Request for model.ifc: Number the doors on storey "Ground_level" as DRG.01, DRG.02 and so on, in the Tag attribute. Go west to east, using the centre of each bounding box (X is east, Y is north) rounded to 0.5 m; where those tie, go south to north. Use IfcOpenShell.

First a look at what the model holds.

```python
import ifcopenshell
import ifcopenshell.util.element
import ifcopenshell.util.placement

model = ifcopenshell.open("model.ifc")
print(model.schema)
storey = next(s for s in model.by_type("IfcBuildingStorey") if s.Name == "Ground_level")
doors = [e for e in ifcopenshell.util.element.get_decomposition(storey) if e.is_a("IfcDoor")]
for e in sorted(doors, key=lambda e: e.id()):
    origin = ifcopenshell.util.placement.get_local_placement(e.ObjectPlacement)[:3, 3]
    print(e.id(), e.Tag, e.Name, origin.round(2) + 0.0, sep=" | ")
```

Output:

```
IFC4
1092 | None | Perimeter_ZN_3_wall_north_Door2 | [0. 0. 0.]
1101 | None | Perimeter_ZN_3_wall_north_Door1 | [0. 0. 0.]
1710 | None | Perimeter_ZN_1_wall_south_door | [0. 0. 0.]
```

```python
import ifcopenshell
import ifcopenshell.geom
import ifcopenshell.util.element
import ifcopenshell.util.shape

model = ifcopenshell.open("model.ifc")
settings = ifcopenshell.geom.settings()
settings.set("use-world-coords", True)


def centre(element):
    shape = ifcopenshell.geom.create_shape(settings, element)
    return ifcopenshell.util.shape.get_bbox_centroid(shape.geometry)


storey = next(s for s in model.by_type("IfcBuildingStorey") if s.Name == "Ground_level")
doors = [e for e in ifcopenshell.util.element.get_decomposition(storey) if e.is_a("IfcDoor")]

# Insertion points can sit at a corner or the storey origin, so sort by the geometry (in metres).
centres = {e: centre(e) for e in doors}
doors.sort(key=lambda e: (round(centres[e][0] / 0.5), centres[e][1]))

for i, e in enumerate(doors, start=1):
    number = f"DRG.{i:02d}"
    e.Tag = number
    print(e.id(), number)

model.write("model-out.ifc")
```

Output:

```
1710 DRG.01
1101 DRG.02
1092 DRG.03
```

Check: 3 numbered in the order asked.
